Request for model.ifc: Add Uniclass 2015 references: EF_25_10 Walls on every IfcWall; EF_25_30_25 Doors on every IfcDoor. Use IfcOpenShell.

First a look at what the model holds.

```python
import ifcopenshell

model = ifcopenshell.open("model.ifc")
print(model.schema)
print("classifications:", [c.Name for c in model.by_type("IfcClassification")])
for ifc_class in ("IfcDoor", "IfcRoof", "IfcStair", "IfcWall", "IfcWindow"):
    print(ifc_class, len(model.by_type(ifc_class)))
```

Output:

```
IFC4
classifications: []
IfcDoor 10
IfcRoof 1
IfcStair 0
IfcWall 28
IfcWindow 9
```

```python
import ifcopenshell
import ifcopenshell.api.classification

model = ifcopenshell.open("model.ifc")

system = ifcopenshell.api.classification.add_classification(model, classification="Uniclass 2015")

codes = {
    "IfcWall": ("EF_25_10", "Walls"),
    "IfcDoor": ("EF_25_30_25", "Doors"),
}
for ifc_class, (code, name) in codes.items():
    products = model.by_type(ifc_class)
    ifcopenshell.api.classification.add_reference(
        model, products=products, classification=system, identification=code, name=name
    )
    print(code, len(products))

model.write("model_updated.ifc")
```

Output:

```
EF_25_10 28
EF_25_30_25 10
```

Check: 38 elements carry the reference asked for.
